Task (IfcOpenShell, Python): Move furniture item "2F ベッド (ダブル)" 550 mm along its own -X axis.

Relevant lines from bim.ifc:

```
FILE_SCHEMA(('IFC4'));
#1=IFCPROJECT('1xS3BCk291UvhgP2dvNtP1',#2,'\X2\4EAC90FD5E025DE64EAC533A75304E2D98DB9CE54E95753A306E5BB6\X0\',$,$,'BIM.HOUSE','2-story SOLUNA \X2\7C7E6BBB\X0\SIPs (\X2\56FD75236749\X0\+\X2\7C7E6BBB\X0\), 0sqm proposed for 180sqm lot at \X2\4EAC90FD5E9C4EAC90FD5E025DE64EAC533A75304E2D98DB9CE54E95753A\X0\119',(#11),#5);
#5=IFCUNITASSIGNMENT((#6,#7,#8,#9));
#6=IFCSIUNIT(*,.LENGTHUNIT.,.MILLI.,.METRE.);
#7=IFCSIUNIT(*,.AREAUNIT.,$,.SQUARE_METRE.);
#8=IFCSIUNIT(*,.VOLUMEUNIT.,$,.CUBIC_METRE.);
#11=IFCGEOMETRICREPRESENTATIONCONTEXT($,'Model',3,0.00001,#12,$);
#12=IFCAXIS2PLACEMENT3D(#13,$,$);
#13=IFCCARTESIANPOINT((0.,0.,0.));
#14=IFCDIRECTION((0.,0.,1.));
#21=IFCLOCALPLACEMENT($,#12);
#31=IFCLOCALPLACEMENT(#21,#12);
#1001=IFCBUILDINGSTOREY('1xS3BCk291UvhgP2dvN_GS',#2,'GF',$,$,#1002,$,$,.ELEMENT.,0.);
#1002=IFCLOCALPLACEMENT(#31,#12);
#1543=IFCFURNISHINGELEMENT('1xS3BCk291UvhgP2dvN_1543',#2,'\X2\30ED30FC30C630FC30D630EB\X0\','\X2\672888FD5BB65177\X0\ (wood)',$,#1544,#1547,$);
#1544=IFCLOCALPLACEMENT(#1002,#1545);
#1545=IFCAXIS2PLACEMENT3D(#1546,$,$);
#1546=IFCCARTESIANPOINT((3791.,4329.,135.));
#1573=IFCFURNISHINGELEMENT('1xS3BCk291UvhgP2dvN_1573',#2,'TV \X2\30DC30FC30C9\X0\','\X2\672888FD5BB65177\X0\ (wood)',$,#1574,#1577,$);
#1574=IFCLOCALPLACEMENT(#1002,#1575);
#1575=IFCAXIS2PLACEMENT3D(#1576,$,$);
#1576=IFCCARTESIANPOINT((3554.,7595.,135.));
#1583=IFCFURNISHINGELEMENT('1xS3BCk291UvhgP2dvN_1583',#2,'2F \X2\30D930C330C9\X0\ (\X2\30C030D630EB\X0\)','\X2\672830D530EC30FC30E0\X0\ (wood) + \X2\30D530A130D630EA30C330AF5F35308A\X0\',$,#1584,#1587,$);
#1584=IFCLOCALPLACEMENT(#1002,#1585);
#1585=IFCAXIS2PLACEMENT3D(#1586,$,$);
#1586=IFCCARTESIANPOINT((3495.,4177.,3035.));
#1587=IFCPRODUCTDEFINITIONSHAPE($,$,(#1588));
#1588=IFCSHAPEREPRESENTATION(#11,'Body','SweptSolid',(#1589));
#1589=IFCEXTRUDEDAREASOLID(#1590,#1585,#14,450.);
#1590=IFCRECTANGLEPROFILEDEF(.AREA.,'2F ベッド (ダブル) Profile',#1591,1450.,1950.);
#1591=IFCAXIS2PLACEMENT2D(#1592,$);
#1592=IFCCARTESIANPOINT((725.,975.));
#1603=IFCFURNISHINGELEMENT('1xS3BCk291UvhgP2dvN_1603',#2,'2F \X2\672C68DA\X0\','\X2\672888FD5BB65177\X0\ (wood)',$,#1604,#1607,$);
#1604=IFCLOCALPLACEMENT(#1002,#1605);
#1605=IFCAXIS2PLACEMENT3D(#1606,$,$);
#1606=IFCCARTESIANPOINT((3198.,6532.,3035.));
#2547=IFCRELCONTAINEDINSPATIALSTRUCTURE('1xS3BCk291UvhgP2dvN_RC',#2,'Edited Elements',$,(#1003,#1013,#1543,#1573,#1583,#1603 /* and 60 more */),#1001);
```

```python
import ifcopenshell
import ifcopenshell.api.geometry
import ifcopenshell.util.placement

model = ifcopenshell.open("bim.ifc")

item = model.by_id(1583)
matrix = ifcopenshell.util.placement.get_local_placement(item.ObjectPlacement)
matrix[:3, 3] -= matrix[:3, 0] * 550.0
ifcopenshell.api.geometry.edit_object_placement(model, product=item, matrix=matrix, is_si=False)

print(ifcopenshell.util.placement.get_local_placement(item.ObjectPlacement).round(3) + 0.0)

model.write("bim_rev.ifc")
```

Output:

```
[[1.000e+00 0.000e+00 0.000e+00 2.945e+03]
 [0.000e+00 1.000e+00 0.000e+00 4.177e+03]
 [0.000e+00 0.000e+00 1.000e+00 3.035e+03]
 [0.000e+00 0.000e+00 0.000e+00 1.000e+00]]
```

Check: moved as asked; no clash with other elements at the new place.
